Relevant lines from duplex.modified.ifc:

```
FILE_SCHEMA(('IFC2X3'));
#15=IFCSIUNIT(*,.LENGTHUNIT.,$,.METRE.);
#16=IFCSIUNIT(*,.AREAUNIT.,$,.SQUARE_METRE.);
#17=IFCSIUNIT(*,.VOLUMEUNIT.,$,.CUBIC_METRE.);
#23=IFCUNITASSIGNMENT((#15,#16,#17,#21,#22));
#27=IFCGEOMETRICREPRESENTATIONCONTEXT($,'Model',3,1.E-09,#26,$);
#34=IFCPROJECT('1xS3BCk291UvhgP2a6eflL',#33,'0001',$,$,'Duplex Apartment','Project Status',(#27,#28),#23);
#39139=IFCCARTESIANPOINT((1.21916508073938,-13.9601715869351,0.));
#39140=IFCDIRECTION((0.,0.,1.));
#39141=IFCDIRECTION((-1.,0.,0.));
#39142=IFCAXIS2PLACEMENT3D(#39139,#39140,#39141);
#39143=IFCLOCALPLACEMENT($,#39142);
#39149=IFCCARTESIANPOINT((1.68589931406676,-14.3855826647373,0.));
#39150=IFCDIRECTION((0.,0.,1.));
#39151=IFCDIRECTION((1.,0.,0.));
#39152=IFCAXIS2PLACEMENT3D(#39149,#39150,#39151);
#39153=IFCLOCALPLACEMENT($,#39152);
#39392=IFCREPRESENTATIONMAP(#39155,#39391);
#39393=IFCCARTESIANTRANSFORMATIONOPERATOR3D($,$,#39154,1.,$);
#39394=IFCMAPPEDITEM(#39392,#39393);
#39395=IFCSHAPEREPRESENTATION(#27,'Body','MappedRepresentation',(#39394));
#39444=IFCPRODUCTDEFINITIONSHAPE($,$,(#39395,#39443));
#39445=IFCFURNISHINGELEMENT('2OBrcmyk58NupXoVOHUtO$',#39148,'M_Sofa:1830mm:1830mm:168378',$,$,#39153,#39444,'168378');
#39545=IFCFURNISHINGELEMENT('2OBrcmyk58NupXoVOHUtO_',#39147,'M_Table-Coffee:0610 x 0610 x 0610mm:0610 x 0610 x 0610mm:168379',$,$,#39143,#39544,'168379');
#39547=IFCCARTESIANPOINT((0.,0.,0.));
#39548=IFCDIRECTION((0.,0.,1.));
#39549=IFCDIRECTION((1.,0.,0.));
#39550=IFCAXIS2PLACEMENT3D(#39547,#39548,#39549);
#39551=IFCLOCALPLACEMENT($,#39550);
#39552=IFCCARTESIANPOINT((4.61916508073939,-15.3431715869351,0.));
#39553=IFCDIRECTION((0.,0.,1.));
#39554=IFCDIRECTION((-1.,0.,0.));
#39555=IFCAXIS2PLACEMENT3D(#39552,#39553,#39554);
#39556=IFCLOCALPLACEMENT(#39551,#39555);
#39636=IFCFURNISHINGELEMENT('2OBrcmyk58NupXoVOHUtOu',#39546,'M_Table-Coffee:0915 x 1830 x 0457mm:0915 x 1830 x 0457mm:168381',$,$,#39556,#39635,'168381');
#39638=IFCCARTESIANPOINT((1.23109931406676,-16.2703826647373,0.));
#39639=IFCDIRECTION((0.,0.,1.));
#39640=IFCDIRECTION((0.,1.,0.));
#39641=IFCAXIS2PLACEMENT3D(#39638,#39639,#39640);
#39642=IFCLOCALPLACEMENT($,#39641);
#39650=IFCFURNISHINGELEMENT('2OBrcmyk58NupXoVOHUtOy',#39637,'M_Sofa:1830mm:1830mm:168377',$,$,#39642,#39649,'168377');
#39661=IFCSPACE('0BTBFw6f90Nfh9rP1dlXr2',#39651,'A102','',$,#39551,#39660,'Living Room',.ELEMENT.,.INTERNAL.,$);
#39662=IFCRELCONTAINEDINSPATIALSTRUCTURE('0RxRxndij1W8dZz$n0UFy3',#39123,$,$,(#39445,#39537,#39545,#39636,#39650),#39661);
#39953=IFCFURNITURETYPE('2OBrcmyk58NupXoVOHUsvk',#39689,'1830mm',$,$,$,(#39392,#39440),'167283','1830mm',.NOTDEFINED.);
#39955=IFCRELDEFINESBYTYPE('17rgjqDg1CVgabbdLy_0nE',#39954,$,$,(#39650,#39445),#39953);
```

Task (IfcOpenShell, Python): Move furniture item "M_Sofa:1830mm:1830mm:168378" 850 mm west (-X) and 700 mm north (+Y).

```python
import ifcopenshell
import ifcopenshell.api.geometry
import ifcopenshell.util.placement

model = ifcopenshell.open("duplex.modified.ifc")

item = model.by_guid("2OBrcmyk58NupXoVOHUtO$")
matrix = ifcopenshell.util.placement.get_local_placement(item.ObjectPlacement)
matrix[0, 3] -= 0.85
matrix[1, 3] += 0.7
ifcopenshell.api.geometry.edit_object_placement(model, product=item, matrix=matrix, is_si=False)

print(ifcopenshell.util.placement.get_local_placement(item.ObjectPlacement).round(3) + 0.0)

model.write("duplex.modified_updated.ifc")
```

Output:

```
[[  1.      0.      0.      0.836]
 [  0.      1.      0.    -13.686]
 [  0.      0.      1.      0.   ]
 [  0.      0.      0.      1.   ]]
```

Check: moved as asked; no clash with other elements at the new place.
